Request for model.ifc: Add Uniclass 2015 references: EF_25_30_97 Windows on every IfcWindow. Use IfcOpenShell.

First a look at what the model holds.

```python
import ifcopenshell

model = ifcopenshell.open("model.ifc")
print(model.schema)
print("classifications:", [c.Name for c in model.by_type("IfcClassification")])
for ifc_class in ("IfcDoor", "IfcRoof", "IfcStair", "IfcWall", "IfcWindow"):
    print(ifc_class, len(model.by_type(ifc_class)))
```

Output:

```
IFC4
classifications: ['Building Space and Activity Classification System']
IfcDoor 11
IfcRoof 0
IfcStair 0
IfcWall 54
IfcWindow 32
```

```python
import ifcopenshell
import ifcopenshell.api.classification

model = ifcopenshell.open("model.ifc")

system = ifcopenshell.api.classification.add_classification(model, classification="Uniclass 2015")

codes = {
    "IfcWindow": ("EF_25_30_97", "Windows"),
}
for ifc_class, (code, name) in codes.items():
    products = model.by_type(ifc_class)
    ifcopenshell.api.classification.add_reference(
        model, products=products, classification=system, identification=code, name=name
    )
    print(code, len(products))

model.write("model_edited.ifc")
```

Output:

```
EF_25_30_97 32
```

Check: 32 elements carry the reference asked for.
